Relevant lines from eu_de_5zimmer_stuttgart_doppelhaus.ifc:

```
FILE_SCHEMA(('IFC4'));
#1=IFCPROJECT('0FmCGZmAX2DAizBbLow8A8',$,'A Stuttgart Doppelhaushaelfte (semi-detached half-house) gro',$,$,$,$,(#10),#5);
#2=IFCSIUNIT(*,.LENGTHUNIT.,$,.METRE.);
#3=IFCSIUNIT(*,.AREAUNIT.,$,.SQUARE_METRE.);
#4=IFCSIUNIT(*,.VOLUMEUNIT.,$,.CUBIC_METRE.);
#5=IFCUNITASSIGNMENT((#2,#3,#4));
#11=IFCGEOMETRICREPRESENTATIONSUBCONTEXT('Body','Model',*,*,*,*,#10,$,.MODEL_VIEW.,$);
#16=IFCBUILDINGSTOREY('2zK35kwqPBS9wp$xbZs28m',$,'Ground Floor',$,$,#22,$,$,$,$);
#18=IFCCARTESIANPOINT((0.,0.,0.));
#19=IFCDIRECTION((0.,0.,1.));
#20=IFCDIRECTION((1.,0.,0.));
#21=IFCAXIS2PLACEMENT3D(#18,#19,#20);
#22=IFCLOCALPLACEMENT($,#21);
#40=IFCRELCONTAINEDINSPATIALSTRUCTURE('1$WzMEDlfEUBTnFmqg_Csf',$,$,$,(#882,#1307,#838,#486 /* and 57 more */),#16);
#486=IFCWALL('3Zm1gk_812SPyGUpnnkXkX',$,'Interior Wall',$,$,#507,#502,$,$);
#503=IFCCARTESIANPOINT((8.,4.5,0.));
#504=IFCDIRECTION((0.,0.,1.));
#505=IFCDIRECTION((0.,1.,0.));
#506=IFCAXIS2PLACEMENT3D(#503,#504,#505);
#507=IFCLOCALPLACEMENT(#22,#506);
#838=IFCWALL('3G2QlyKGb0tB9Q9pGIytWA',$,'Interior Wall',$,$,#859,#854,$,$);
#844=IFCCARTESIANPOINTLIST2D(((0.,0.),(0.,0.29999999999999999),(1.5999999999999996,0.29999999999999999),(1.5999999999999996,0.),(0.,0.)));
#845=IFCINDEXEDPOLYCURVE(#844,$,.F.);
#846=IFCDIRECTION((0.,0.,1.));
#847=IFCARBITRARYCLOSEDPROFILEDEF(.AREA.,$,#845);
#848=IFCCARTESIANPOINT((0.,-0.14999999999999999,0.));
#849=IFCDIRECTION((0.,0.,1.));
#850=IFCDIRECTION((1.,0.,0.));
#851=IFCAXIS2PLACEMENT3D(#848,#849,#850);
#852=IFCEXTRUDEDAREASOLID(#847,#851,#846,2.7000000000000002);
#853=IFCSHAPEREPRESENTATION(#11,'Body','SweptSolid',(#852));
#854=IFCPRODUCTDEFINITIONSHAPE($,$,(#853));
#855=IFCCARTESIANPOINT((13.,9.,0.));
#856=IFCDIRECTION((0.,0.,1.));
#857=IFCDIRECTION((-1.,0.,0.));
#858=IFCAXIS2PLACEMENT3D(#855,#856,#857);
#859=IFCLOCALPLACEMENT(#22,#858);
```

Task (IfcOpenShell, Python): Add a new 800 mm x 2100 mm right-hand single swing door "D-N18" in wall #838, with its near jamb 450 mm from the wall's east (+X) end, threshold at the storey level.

```python
import numpy as np
import ifcopenshell
import ifcopenshell.api.feature
import ifcopenshell.api.geometry
import ifcopenshell.api.root
import ifcopenshell.api.spatial
import ifcopenshell.geom
import ifcopenshell.util.element
import ifcopenshell.util.placement
import ifcopenshell.util.representation
import ifcopenshell.util.shape
import ifcopenshell.util.unit

model = ifcopenshell.open("eu_de_5zimmer_stuttgart_doppelhaus.ifc")
unit_scale = ifcopenshell.util.unit.calculate_unit_scale(model)
settings = ifcopenshell.geom.settings()


def volume(element):
    """Net volume in cubic metres, openings subtracted."""
    shape = ifcopenshell.geom.create_shape(settings, element)
    return ifcopenshell.util.shape.get_volume(shape.geometry)


wall = model.by_id(838)
storey = ifcopenshell.util.element.get_container(wall, ifc_class="IfcBuildingStorey")
context = ifcopenshell.util.representation.get_context(model, "Model", "Body", "MODEL_VIEW")
before = volume(wall)

width, height, from_end, sill = 0.8, 2.1, 0.45, 0.0  # metres

# The wall runs along its own X axis, and the end named is its -X end.
wall_shape = ifcopenshell.geom.create_shape(settings, wall)
x, y, z = ifcopenshell.util.shape.get_vertices(wall_shape.geometry).T
start = x.min() + from_end
face, thickness = float(y.min()), float(y.max() - y.min())
wall_matrix = ifcopenshell.util.placement.get_local_placement(wall.ObjectPlacement)
level = ifcopenshell.util.placement.get_local_placement(storey.ObjectPlacement)[2, 3]


def in_wall(x, y):
    """Placement at x, y metres in the wall's axes, at sill height."""
    matrix = wall_matrix.copy()
    matrix[:, 3] = wall_matrix @ np.array([x / unit_scale, y / unit_scale, 0.0, 1.0])
    matrix[2, 3] = level + sill / unit_scale
    return matrix


# Opening: a box that overshoots both wall faces by 50 mm.
opening = ifcopenshell.api.root.create_entity(model, ifc_class="IfcOpeningElement", predefined_type="OPENING")
box = ifcopenshell.api.geometry.add_wall_representation(
    model, context=context, length=width, height=height, thickness=thickness + 0.1
)
ifcopenshell.api.geometry.assign_representation(model, product=opening, representation=box)
ifcopenshell.api.geometry.edit_object_placement(model, product=opening, matrix=in_wall(start, face - 0.05), is_si=False)
ifcopenshell.api.feature.add_feature(model, feature=opening, element=wall)

door = ifcopenshell.api.root.create_entity(model, ifc_class="IfcDoor", name="D-N18", predefined_type="DOOR")
door.OverallWidth, door.OverallHeight = width / unit_scale, height / unit_scale
door.OperationType = "SINGLE_SWING_RIGHT"
body = ifcopenshell.api.geometry.add_door_representation(
    model,
    context=context,
    overall_width=door.OverallWidth,
    overall_height=door.OverallHeight,
    operation_type="SINGLE_SWING_RIGHT",
    lining_properties={"LiningDepth": thickness / unit_scale, "ThresholdDepth": thickness / unit_scale},
)
ifcopenshell.api.geometry.assign_representation(model, product=door, representation=body)
ifcopenshell.api.spatial.assign_container(model, products=[door], relating_structure=storey)
ifcopenshell.api.feature.add_filling(model, opening=opening, element=door)

# The lining spans the wall, so the door starts at the wall face.
ifcopenshell.api.geometry.edit_object_placement(model, product=door, matrix=in_wall(start, face), is_si=False)

after = volume(wall)

print(f"wall volume {before:.3f} -> {after:.3f} m3")

model.write("eu_de_5zimmer_stuttgart_doppelhaus_v2.ifc")
```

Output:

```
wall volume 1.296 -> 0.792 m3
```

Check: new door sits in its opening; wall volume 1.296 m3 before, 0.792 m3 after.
